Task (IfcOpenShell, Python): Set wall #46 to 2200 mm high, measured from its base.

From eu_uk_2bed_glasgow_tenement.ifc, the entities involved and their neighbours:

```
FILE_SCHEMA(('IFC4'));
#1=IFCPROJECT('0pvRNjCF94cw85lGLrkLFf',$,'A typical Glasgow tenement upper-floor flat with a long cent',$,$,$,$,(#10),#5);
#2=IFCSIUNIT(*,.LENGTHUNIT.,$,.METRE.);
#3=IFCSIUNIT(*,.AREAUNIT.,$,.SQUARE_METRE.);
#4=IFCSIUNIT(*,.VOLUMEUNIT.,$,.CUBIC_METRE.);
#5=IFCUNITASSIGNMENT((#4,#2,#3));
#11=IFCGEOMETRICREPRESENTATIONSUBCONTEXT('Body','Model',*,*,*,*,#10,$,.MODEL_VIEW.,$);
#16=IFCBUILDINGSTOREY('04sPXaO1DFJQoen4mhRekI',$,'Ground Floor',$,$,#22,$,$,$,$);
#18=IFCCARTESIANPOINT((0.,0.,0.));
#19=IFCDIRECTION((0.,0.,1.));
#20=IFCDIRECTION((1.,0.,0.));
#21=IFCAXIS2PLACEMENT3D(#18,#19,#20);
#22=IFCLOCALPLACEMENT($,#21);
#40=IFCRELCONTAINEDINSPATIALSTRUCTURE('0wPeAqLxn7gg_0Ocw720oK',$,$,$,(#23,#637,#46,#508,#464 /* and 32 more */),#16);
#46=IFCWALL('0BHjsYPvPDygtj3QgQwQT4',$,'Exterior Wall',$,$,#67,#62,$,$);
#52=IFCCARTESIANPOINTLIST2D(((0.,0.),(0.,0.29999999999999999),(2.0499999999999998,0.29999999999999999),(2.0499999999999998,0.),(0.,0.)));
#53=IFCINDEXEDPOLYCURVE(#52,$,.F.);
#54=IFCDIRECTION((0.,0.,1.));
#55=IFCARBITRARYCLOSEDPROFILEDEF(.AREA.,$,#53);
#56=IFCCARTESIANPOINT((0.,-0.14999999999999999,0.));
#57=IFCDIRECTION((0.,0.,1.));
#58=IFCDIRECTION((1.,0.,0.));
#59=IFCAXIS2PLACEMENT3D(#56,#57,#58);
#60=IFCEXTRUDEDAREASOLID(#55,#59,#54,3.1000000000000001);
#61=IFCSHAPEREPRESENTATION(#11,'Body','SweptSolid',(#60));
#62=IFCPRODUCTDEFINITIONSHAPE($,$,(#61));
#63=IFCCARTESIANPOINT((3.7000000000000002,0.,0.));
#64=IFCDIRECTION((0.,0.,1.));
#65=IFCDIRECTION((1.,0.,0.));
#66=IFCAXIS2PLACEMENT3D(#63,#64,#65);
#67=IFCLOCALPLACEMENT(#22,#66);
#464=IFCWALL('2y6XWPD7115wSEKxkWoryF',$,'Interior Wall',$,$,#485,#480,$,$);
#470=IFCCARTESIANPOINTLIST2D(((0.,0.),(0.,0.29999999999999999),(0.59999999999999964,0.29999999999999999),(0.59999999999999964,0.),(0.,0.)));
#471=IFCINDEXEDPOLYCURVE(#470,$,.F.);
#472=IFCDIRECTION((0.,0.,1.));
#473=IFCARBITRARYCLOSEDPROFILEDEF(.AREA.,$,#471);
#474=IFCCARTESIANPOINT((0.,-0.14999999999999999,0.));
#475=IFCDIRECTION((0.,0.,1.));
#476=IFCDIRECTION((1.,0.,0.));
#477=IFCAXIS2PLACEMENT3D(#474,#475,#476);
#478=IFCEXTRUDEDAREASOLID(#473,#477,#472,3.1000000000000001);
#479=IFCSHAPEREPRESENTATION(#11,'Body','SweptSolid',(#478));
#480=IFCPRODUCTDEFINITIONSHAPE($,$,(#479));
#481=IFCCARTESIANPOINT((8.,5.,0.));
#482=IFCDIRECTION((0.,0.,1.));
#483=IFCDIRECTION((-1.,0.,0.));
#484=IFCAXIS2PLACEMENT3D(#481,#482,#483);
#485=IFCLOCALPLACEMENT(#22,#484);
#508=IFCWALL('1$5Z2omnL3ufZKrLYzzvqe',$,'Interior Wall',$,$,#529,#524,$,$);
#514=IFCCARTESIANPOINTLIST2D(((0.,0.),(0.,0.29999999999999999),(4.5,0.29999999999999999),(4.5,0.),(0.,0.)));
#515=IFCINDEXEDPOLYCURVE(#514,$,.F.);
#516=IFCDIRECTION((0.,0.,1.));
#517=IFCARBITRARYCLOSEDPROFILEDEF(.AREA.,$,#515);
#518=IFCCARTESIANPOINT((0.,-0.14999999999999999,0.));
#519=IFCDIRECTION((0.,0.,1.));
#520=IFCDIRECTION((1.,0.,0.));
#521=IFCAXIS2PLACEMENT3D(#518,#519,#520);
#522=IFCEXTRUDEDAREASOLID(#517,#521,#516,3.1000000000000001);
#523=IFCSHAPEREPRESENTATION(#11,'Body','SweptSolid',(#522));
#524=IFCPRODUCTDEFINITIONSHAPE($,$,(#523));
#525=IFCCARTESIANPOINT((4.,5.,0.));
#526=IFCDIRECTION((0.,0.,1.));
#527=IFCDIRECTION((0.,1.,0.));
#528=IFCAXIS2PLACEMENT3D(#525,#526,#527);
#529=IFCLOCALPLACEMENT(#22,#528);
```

```python
import ifcopenshell
import ifcopenshell.geom
import ifcopenshell.util.representation
import ifcopenshell.util.shape

model = ifcopenshell.open("eu_uk_2bed_glasgow_tenement.ifc")
settings = ifcopenshell.geom.settings()


def volume(element):
    """Net volume in cubic metres, openings subtracted."""
    shape = ifcopenshell.geom.create_shape(settings, element)
    return ifcopenshell.util.shape.get_volume(shape.geometry)


wall = model.by_guid("0BHjsYPvPDygtj3QgQwQT4")
before = volume(wall)

body = ifcopenshell.util.representation.get_representation(wall, "Model", "Body")
solid = body.Items[0]
old_height = solid.Depth
solid.Depth = 2.2
after = volume(wall)

print(f"height {old_height:g} -> {solid.Depth:g}, volume {before:.3f} -> {after:.3f} m3")

model.write("eu_uk_2bed_glasgow_tenement-out.ifc")
```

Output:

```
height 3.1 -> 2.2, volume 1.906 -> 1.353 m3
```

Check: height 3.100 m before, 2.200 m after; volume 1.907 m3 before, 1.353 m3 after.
